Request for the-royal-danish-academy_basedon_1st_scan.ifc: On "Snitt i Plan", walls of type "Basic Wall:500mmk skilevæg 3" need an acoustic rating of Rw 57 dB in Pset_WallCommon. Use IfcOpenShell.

First a look at what the model holds.

```python
import ifcopenshell
import ifcopenshell.util.element

model = ifcopenshell.open("the-royal-danish-academy_basedon_1st_scan.ifc")
print(model.schema)
storey = next(s for s in model.by_type("IfcBuildingStorey") if s.Name == "Snitt i Plan")
walls = [e for e in ifcopenshell.util.element.get_decomposition(storey) if e.is_a("IfcWall")]
seen = {}
for e in walls:
    element_type = ifcopenshell.util.element.get_type(e)
    key = (element_type.Name if element_type != e and element_type else None, ifcopenshell.util.element.get_pset(e, "Pset_WallCommon", "AcousticRating"))
    seen[key] = seen.get(key, 0) + 1
for (name, value), count in sorted(seen.items(), key=str):
    print(count, "x", name, "|", value)
```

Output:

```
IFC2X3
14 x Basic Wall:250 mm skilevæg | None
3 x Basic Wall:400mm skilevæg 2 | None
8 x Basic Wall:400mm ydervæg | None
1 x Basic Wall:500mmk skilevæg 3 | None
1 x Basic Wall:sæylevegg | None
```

```python
import ifcopenshell
import ifcopenshell.api.pset
import ifcopenshell.util.element

model = ifcopenshell.open("the-royal-danish-academy_basedon_1st_scan.ifc")

storey = next(s for s in model.by_type("IfcBuildingStorey") if s.Name == "Snitt i Plan")
walls = [e for e in ifcopenshell.util.element.get_decomposition(storey) if e.is_a("IfcWall")]

count = 0
for e in walls:
    element_type = ifcopenshell.util.element.get_type(e)
    if element_type in (None, e) or element_type.Name != "Basic Wall:500mmk skilevæg 3":
        continue
    # add_pset returns the element's existing set when there is one.
    pset = ifcopenshell.api.pset.add_pset(model, product=e, name="Pset_WallCommon")
    ifcopenshell.api.pset.edit_pset(model, pset=pset, properties={"AcousticRating": "Rw 57 dB"})
    count += 1

print(count, "walls updated")

model.write("the-royal-danish-academy_basedon_1st_scan_edited.ifc")
```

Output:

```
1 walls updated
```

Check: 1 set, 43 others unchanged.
